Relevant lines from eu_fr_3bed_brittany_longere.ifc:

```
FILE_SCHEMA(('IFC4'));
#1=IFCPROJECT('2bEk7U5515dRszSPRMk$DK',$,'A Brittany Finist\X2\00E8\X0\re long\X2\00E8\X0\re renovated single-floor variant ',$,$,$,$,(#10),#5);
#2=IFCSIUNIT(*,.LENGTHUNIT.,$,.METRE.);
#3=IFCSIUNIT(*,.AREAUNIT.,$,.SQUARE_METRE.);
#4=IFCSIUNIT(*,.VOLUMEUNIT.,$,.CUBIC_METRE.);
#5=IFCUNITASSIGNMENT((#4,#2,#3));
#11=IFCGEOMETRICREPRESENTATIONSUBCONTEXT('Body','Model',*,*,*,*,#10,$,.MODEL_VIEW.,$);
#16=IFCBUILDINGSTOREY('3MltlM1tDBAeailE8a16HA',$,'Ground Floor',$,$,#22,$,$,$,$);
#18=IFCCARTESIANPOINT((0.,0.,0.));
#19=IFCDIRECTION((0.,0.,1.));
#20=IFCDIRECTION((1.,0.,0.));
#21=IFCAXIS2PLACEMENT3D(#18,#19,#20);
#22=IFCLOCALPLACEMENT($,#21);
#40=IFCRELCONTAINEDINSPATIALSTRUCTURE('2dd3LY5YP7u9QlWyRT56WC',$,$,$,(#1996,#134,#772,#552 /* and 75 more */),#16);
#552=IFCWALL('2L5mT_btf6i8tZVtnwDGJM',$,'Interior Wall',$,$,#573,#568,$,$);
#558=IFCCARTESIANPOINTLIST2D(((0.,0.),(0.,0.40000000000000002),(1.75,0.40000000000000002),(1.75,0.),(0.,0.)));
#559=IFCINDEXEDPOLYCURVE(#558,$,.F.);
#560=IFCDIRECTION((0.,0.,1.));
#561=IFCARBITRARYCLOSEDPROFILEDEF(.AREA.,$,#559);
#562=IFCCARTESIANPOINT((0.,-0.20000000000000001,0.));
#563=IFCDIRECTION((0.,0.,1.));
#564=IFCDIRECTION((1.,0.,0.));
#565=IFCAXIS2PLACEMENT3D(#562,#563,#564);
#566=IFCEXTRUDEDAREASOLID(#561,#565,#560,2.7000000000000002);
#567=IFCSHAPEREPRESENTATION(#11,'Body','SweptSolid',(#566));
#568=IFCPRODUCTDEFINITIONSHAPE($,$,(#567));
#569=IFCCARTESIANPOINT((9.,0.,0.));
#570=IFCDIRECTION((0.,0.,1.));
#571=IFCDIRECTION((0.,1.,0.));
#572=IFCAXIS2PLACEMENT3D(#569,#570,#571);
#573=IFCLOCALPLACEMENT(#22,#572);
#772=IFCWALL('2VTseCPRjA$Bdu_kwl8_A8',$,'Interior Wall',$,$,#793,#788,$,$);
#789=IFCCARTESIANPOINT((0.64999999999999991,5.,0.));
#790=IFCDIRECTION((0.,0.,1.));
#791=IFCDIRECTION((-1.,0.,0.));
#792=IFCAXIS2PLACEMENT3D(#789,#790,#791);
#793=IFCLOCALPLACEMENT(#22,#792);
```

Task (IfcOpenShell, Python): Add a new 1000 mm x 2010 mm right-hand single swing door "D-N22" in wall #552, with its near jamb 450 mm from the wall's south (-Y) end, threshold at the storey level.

```python
import numpy as np
import ifcopenshell
import ifcopenshell.api.feature
import ifcopenshell.api.geometry
import ifcopenshell.api.root
import ifcopenshell.api.spatial
import ifcopenshell.geom
import ifcopenshell.util.element
import ifcopenshell.util.placement
import ifcopenshell.util.representation
import ifcopenshell.util.shape
import ifcopenshell.util.unit

model = ifcopenshell.open("eu_fr_3bed_brittany_longere.ifc")
unit_scale = ifcopenshell.util.unit.calculate_unit_scale(model)
settings = ifcopenshell.geom.settings()


def volume(element):
    """Net volume in cubic metres, openings subtracted."""
    shape = ifcopenshell.geom.create_shape(settings, element)
    return ifcopenshell.util.shape.get_volume(shape.geometry)


wall = model.by_id(552)
storey = ifcopenshell.util.element.get_container(wall, ifc_class="IfcBuildingStorey")
context = ifcopenshell.util.representation.get_context(model, "Model", "Body", "MODEL_VIEW")
before = volume(wall)

width, height, from_end, sill = 1, 2.01, 0.45, 0.0  # metres

# The wall runs along its own X axis, and the end named is its -X end.
wall_shape = ifcopenshell.geom.create_shape(settings, wall)
x, y, z = ifcopenshell.util.shape.get_vertices(wall_shape.geometry).T
start = x.min() + from_end
face, thickness = float(y.min()), float(y.max() - y.min())
wall_matrix = ifcopenshell.util.placement.get_local_placement(wall.ObjectPlacement)
level = ifcopenshell.util.placement.get_local_placement(storey.ObjectPlacement)[2, 3]


def in_wall(x, y):
    """Placement at x, y metres in the wall's axes, at sill height."""
    matrix = wall_matrix.copy()
    matrix[:, 3] = wall_matrix @ np.array([x / unit_scale, y / unit_scale, 0.0, 1.0])
    matrix[2, 3] = level + sill / unit_scale
    return matrix


# Opening: a box that overshoots both wall faces by 50 mm.
opening = ifcopenshell.api.root.create_entity(model, ifc_class="IfcOpeningElement", predefined_type="OPENING")
box = ifcopenshell.api.geometry.add_wall_representation(
    model, context=context, length=width, height=height, thickness=thickness + 0.1
)
ifcopenshell.api.geometry.assign_representation(model, product=opening, representation=box)
ifcopenshell.api.geometry.edit_object_placement(model, product=opening, matrix=in_wall(start, face - 0.05), is_si=False)
ifcopenshell.api.feature.add_feature(model, feature=opening, element=wall)

door = ifcopenshell.api.root.create_entity(model, ifc_class="IfcDoor", name="D-N22", predefined_type="DOOR")
door.OverallWidth, door.OverallHeight = width / unit_scale, height / unit_scale
door.OperationType = "SINGLE_SWING_RIGHT"
body = ifcopenshell.api.geometry.add_door_representation(
    model,
    context=context,
    overall_width=door.OverallWidth,
    overall_height=door.OverallHeight,
    operation_type="SINGLE_SWING_RIGHT",
    lining_properties={"LiningDepth": thickness / unit_scale, "ThresholdDepth": thickness / unit_scale},
)
ifcopenshell.api.geometry.assign_representation(model, product=door, representation=body)
ifcopenshell.api.spatial.assign_container(model, products=[door], relating_structure=storey)
ifcopenshell.api.feature.add_filling(model, opening=opening, element=door)

# The lining spans the wall, so the door starts at the wall face.
ifcopenshell.api.geometry.edit_object_placement(model, product=door, matrix=in_wall(start, face), is_si=False)

after = volume(wall)

print(f"wall volume {before:.3f} -> {after:.3f} m3")

model.write("eu_fr_3bed_brittany_longere_updated.ifc")
```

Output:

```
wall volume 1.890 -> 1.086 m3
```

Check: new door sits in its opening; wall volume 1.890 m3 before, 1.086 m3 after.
